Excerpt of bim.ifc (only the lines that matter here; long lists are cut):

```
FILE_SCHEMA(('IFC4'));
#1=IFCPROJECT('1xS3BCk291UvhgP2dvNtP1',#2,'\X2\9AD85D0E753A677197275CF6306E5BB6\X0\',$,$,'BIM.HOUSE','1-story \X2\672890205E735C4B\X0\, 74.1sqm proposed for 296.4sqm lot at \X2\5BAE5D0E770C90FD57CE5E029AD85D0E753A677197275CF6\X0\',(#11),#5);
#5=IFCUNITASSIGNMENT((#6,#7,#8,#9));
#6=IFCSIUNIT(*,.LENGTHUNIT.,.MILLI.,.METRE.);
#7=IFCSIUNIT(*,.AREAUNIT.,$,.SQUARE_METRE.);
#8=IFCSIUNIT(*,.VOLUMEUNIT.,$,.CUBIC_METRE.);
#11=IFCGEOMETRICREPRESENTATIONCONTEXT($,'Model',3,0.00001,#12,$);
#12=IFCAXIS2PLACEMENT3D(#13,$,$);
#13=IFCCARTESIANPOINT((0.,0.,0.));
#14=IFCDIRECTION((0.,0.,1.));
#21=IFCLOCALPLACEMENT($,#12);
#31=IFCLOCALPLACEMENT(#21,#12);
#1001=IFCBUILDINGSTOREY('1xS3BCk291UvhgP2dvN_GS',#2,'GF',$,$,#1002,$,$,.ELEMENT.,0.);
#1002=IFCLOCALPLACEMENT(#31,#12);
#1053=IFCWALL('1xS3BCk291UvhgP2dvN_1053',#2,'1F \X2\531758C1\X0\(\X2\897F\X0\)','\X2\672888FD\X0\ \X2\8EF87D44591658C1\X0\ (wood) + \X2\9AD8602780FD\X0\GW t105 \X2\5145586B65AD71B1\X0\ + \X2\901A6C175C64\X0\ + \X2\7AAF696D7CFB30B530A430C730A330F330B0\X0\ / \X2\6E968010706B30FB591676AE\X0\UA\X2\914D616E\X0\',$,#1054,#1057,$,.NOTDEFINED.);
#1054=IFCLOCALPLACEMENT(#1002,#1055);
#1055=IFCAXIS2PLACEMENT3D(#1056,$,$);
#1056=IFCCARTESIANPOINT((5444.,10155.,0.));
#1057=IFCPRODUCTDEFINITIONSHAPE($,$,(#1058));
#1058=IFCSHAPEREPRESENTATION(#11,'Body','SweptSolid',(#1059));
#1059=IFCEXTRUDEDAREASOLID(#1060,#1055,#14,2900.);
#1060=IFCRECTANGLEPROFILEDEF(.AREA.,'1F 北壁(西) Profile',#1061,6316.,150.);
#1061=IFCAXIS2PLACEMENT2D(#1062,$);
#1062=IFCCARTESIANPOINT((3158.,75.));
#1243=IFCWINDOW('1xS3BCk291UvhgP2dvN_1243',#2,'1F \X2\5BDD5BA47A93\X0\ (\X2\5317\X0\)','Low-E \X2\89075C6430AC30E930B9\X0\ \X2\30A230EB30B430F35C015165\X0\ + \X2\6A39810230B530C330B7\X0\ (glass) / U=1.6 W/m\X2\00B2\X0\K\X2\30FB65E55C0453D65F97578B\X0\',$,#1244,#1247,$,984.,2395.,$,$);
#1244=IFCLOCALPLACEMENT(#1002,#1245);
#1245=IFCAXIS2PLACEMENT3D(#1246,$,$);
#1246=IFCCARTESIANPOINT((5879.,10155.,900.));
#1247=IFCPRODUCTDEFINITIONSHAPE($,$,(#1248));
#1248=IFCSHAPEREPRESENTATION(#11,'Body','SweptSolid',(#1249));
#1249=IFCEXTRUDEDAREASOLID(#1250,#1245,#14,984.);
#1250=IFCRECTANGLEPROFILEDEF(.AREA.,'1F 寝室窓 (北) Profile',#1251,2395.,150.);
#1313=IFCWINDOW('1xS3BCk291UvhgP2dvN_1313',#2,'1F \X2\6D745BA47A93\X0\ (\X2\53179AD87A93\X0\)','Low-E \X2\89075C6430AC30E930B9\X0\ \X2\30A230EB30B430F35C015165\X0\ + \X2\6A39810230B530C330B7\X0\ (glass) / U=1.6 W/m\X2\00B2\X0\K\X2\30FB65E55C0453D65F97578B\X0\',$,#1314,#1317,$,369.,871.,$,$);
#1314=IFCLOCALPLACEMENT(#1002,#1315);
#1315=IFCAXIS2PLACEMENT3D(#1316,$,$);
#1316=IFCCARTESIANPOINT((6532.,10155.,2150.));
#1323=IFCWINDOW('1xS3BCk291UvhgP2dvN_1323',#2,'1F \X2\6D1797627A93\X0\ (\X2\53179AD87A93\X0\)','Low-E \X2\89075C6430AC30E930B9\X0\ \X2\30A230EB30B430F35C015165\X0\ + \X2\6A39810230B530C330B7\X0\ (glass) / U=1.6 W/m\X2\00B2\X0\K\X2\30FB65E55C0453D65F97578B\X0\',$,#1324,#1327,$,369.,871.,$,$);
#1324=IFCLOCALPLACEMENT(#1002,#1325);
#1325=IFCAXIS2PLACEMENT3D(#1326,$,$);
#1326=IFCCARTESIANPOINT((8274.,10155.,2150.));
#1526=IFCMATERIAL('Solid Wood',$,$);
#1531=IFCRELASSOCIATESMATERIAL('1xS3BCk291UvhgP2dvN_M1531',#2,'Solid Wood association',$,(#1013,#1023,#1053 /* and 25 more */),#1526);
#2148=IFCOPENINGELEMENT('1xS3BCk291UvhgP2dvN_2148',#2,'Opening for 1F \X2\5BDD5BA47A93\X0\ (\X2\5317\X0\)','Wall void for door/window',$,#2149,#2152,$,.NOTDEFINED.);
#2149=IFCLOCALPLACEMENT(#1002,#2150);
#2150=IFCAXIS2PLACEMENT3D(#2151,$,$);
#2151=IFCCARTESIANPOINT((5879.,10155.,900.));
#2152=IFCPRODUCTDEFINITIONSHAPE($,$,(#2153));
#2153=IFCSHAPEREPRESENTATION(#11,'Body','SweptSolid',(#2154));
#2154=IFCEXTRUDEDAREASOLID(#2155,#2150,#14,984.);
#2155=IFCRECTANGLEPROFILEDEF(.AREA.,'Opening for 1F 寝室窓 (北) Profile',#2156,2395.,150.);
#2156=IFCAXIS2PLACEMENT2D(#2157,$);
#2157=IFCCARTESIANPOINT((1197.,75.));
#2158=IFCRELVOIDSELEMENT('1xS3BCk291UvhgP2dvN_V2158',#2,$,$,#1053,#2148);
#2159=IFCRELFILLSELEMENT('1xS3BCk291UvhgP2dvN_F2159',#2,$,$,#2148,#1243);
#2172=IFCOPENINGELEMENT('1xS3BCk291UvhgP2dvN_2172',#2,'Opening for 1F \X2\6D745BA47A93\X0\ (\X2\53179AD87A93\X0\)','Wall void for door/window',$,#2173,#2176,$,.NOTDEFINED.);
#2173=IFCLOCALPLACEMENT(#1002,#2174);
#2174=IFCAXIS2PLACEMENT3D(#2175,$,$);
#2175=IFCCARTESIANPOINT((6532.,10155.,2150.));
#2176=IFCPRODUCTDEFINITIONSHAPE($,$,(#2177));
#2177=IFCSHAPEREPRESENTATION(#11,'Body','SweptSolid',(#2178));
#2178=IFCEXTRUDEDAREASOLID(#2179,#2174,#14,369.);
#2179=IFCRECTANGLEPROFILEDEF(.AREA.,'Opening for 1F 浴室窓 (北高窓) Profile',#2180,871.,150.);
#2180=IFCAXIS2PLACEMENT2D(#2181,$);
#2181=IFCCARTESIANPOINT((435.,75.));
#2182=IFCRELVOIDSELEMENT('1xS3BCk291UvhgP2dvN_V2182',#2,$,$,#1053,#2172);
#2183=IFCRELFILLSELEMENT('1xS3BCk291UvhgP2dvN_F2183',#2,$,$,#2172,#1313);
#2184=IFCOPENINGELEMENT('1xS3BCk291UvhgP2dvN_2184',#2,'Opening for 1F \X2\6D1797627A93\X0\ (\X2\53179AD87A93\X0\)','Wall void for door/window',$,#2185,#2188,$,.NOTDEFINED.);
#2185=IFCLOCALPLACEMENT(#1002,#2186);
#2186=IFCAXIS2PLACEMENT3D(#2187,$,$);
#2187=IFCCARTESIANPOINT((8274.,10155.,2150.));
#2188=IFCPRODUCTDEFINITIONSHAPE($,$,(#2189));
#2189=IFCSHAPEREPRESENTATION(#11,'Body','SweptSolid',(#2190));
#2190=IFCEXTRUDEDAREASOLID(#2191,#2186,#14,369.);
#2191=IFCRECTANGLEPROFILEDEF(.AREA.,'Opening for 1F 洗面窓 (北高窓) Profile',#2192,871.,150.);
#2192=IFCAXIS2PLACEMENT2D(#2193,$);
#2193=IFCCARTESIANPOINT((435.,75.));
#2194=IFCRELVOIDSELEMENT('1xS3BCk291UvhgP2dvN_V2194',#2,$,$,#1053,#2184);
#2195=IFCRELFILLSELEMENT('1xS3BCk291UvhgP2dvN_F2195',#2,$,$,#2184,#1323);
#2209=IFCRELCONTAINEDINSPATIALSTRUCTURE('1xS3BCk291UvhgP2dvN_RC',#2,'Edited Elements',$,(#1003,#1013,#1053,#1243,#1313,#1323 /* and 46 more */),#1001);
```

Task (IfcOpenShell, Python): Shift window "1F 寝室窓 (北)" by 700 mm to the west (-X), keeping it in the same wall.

```python
import ifcopenshell
import ifcopenshell.api.geometry
import ifcopenshell.util.placement

model = ifcopenshell.open("bim.ifc")

window = model.by_guid("1xS3BCk291UvhgP2dvN_1243")
opening = window.FillsVoids[0].RelatingOpeningElement
wall = opening.VoidsElements[0].RelatingBuildingElement

wall_matrix = ifcopenshell.util.placement.get_local_placement(wall.ObjectPlacement)
shift = wall_matrix[:3, 0] * -700.0
before = ifcopenshell.util.placement.get_local_placement(window.ObjectPlacement)[:3, 3].copy()

# The window is not placed relative to its opening, so move both.
for product in (opening, window):
    matrix = ifcopenshell.util.placement.get_local_placement(product.ObjectPlacement)
    matrix[:3, 3] += shift
    ifcopenshell.api.geometry.edit_object_placement(model, product=product, matrix=matrix, is_si=False)

after = ifcopenshell.util.placement.get_local_placement(window.ObjectPlacement)[:3, 3]
print("window moved by", (after - before).round(3) + 0.0)

model.write("bim_edited.ifc")
```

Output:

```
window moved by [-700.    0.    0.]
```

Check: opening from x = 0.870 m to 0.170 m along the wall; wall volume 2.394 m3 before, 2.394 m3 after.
